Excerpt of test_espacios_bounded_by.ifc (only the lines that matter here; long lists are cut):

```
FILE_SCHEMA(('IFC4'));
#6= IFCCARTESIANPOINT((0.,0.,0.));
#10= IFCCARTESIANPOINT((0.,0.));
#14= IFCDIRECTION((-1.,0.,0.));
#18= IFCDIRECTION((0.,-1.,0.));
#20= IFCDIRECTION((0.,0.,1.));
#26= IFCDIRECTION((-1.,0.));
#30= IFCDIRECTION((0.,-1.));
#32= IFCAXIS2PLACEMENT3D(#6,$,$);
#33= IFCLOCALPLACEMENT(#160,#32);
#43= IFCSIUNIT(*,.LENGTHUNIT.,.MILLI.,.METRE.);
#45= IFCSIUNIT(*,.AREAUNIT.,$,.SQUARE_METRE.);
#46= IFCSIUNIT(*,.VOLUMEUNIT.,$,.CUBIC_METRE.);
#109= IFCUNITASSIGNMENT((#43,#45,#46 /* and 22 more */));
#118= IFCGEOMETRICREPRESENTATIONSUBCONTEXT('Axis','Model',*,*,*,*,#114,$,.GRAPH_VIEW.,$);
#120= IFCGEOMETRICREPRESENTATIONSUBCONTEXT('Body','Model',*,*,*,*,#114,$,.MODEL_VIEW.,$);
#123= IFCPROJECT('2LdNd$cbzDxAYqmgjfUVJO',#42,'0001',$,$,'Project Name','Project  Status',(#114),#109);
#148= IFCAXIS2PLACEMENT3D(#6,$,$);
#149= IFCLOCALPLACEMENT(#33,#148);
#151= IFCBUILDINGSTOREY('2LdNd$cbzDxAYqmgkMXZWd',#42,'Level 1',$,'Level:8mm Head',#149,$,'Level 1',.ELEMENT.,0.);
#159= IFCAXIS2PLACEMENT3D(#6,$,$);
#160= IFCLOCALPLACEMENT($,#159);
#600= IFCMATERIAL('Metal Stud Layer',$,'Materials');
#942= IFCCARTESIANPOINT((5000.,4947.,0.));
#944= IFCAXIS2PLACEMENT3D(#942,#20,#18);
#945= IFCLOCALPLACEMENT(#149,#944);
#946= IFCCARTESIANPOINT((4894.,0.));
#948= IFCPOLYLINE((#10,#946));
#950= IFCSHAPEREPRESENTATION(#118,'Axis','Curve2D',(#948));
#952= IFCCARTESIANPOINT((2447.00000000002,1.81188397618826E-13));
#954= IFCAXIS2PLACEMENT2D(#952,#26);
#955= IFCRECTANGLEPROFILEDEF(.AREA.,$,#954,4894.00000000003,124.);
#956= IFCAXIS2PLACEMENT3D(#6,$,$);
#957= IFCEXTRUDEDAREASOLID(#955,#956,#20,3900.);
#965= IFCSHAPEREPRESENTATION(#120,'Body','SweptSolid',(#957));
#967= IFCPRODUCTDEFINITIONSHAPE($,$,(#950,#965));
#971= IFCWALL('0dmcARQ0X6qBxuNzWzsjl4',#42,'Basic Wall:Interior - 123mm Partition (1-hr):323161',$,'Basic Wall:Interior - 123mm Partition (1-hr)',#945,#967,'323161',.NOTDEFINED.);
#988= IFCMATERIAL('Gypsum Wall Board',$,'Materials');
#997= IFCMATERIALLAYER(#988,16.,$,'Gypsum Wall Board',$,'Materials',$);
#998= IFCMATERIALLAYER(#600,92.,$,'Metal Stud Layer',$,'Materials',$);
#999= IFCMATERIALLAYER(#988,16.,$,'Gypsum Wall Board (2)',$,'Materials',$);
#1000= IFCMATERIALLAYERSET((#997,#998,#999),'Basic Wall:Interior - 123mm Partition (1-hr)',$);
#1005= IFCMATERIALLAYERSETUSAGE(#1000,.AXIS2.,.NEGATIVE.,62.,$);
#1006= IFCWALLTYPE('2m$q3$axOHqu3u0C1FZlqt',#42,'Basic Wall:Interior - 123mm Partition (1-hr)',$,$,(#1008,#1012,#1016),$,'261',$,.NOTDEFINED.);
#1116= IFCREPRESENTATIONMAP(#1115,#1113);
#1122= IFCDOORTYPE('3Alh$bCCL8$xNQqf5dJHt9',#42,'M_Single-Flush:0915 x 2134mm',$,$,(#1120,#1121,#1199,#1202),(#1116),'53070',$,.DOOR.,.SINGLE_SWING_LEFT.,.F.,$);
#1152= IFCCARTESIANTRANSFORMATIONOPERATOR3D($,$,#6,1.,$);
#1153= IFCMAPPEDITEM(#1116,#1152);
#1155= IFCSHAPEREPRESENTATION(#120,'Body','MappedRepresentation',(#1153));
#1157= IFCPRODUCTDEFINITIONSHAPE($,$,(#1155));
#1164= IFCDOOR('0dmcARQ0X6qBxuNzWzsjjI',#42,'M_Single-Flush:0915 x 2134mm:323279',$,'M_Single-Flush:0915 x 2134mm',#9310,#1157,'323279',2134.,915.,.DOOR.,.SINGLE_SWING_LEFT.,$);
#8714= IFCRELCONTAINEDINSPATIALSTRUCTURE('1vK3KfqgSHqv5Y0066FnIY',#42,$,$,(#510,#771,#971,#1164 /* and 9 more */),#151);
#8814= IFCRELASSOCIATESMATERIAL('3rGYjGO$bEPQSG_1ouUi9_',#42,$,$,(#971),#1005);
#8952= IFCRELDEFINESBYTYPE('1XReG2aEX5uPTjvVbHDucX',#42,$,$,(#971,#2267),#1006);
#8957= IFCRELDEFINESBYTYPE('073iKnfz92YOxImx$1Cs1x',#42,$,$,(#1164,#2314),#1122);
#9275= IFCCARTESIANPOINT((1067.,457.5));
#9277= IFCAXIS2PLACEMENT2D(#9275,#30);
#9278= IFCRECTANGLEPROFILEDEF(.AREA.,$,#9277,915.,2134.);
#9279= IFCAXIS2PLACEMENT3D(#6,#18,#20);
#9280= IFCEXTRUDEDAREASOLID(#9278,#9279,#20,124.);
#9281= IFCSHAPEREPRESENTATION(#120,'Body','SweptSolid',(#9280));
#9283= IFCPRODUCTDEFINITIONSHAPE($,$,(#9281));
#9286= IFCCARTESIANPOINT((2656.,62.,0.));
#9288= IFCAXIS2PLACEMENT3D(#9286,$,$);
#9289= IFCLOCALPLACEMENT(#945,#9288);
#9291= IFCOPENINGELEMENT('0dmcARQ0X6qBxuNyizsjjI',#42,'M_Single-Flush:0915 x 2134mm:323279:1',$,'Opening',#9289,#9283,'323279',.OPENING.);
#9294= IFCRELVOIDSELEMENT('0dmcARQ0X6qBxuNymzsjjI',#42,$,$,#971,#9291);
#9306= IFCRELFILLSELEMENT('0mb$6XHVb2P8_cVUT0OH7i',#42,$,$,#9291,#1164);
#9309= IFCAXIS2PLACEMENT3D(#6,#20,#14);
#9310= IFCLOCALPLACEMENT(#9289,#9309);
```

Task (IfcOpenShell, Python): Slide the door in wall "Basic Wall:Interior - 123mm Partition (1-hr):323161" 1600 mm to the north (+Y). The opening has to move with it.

```python
import ifcopenshell
import ifcopenshell.api.geometry
import ifcopenshell.util.placement

model = ifcopenshell.open("test_espacios_bounded_by.ifc")

door = model.by_guid("0dmcARQ0X6qBxuNzWzsjjI")
opening = door.FillsVoids[0].RelatingOpeningElement
wall = opening.VoidsElements[0].RelatingBuildingElement

wall_matrix = ifcopenshell.util.placement.get_local_placement(wall.ObjectPlacement)
shift = wall_matrix[:3, 0] * -1600.0
before = ifcopenshell.util.placement.get_local_placement(door.ObjectPlacement)[:3, 3].copy()

# The door is placed relative to its opening, so it follows when the opening moves.
matrix = ifcopenshell.util.placement.get_local_placement(opening.ObjectPlacement)
matrix[:3, 3] += shift
ifcopenshell.api.geometry.edit_object_placement(
    model, product=opening, matrix=matrix, is_si=False, should_transform_children=True
)

after = ifcopenshell.util.placement.get_local_placement(door.ObjectPlacement)[:3, 3]
print("door moved by", (after - before).round(3) + 0.0)

model.write("test_espacios_bounded_by-out.ifc")
```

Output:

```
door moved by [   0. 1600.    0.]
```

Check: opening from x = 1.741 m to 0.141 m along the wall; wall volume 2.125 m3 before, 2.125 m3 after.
